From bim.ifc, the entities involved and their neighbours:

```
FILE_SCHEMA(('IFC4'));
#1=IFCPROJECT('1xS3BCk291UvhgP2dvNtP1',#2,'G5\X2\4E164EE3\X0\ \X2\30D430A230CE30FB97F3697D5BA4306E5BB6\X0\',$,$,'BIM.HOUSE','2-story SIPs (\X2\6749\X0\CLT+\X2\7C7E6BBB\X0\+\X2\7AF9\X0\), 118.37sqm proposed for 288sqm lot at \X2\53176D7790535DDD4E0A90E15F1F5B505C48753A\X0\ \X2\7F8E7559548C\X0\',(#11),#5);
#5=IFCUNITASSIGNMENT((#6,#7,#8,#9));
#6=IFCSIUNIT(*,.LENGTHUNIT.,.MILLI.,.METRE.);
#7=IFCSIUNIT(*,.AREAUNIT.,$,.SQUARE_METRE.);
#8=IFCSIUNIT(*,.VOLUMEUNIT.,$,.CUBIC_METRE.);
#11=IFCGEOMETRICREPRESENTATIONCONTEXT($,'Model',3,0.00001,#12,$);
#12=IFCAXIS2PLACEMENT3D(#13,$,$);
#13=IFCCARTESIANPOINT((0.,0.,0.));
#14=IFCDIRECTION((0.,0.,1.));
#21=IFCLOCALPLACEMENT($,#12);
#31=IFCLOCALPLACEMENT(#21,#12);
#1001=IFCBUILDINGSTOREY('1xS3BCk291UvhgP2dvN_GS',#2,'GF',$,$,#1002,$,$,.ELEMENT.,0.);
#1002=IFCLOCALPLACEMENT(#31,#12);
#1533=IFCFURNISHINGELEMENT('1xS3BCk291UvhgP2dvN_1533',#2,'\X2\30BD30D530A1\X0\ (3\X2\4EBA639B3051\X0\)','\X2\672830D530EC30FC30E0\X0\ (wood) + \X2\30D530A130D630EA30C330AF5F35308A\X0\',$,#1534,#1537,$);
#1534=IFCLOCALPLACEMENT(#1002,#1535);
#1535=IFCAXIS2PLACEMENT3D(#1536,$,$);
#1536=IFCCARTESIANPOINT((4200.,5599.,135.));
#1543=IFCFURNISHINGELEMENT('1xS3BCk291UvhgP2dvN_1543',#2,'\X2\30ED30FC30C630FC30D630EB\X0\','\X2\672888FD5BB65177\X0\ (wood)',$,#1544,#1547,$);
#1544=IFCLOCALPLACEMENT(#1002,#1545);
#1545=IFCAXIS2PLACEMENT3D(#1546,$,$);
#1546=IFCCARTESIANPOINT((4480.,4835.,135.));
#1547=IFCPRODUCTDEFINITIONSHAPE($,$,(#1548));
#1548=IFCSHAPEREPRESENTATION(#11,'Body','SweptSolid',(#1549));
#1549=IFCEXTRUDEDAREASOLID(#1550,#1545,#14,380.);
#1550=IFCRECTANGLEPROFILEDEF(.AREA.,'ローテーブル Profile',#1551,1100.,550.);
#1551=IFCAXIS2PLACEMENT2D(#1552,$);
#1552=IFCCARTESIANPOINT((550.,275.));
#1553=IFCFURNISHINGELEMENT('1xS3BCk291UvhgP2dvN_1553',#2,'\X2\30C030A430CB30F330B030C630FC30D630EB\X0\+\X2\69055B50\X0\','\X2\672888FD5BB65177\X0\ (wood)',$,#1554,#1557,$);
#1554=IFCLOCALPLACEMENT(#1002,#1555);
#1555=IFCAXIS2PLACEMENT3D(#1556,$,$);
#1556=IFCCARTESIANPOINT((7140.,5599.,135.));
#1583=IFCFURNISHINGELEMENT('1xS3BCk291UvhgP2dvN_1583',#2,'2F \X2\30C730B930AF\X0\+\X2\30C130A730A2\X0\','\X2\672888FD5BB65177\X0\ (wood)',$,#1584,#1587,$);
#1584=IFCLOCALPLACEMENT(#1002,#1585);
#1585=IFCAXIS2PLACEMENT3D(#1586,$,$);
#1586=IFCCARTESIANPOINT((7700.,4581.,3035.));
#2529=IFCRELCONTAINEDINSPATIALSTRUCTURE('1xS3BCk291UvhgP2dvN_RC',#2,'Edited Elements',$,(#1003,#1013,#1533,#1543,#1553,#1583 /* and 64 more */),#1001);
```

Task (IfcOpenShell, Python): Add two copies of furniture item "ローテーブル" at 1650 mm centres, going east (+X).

```python
import numpy as np
import ifcopenshell
import ifcopenshell.api.geometry
import ifcopenshell.api.root
import ifcopenshell.util.element
import ifcopenshell.util.placement

model = ifcopenshell.open("bim.ifc")


def reuse_history(source, copy):
    """copy_class also copies each property set's owner history, people and application; keep the originals."""
    for rel in copy.IsDefinedBy:
        if rel.is_a("IfcRelDefinesByProperties") and (history := rel.RelatingPropertyDefinition.OwnerHistory):
            rel.RelatingPropertyDefinition.OwnerHistory = source.OwnerHistory
            ifcopenshell.util.element.remove_deep2(model, history)


source = model.by_id(1543)
base = ifcopenshell.util.placement.get_local_placement(source.ObjectPlacement)
step = np.array([1.0, 0.0, 0.0]) * 1650.0

for i in range(1, 3):
    copy = ifcopenshell.api.root.copy_class(model, product=source)
    copy.Representation = ifcopenshell.util.element.copy_deep(
        model, source.Representation, exclude=["IfcGeometricRepresentationContext", "IfcRepresentationMap"]
    )
    reuse_history(source, copy)
    matrix = base.copy()
    matrix[:3, 3] += i * step
    print("added at", matrix[:3, 3].round(3) + 0.0)
    ifcopenshell.api.geometry.edit_object_placement(model, product=copy, matrix=matrix, is_si=False)

model.write("bim_updated.ifc")
```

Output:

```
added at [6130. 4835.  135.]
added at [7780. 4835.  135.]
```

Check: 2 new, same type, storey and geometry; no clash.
